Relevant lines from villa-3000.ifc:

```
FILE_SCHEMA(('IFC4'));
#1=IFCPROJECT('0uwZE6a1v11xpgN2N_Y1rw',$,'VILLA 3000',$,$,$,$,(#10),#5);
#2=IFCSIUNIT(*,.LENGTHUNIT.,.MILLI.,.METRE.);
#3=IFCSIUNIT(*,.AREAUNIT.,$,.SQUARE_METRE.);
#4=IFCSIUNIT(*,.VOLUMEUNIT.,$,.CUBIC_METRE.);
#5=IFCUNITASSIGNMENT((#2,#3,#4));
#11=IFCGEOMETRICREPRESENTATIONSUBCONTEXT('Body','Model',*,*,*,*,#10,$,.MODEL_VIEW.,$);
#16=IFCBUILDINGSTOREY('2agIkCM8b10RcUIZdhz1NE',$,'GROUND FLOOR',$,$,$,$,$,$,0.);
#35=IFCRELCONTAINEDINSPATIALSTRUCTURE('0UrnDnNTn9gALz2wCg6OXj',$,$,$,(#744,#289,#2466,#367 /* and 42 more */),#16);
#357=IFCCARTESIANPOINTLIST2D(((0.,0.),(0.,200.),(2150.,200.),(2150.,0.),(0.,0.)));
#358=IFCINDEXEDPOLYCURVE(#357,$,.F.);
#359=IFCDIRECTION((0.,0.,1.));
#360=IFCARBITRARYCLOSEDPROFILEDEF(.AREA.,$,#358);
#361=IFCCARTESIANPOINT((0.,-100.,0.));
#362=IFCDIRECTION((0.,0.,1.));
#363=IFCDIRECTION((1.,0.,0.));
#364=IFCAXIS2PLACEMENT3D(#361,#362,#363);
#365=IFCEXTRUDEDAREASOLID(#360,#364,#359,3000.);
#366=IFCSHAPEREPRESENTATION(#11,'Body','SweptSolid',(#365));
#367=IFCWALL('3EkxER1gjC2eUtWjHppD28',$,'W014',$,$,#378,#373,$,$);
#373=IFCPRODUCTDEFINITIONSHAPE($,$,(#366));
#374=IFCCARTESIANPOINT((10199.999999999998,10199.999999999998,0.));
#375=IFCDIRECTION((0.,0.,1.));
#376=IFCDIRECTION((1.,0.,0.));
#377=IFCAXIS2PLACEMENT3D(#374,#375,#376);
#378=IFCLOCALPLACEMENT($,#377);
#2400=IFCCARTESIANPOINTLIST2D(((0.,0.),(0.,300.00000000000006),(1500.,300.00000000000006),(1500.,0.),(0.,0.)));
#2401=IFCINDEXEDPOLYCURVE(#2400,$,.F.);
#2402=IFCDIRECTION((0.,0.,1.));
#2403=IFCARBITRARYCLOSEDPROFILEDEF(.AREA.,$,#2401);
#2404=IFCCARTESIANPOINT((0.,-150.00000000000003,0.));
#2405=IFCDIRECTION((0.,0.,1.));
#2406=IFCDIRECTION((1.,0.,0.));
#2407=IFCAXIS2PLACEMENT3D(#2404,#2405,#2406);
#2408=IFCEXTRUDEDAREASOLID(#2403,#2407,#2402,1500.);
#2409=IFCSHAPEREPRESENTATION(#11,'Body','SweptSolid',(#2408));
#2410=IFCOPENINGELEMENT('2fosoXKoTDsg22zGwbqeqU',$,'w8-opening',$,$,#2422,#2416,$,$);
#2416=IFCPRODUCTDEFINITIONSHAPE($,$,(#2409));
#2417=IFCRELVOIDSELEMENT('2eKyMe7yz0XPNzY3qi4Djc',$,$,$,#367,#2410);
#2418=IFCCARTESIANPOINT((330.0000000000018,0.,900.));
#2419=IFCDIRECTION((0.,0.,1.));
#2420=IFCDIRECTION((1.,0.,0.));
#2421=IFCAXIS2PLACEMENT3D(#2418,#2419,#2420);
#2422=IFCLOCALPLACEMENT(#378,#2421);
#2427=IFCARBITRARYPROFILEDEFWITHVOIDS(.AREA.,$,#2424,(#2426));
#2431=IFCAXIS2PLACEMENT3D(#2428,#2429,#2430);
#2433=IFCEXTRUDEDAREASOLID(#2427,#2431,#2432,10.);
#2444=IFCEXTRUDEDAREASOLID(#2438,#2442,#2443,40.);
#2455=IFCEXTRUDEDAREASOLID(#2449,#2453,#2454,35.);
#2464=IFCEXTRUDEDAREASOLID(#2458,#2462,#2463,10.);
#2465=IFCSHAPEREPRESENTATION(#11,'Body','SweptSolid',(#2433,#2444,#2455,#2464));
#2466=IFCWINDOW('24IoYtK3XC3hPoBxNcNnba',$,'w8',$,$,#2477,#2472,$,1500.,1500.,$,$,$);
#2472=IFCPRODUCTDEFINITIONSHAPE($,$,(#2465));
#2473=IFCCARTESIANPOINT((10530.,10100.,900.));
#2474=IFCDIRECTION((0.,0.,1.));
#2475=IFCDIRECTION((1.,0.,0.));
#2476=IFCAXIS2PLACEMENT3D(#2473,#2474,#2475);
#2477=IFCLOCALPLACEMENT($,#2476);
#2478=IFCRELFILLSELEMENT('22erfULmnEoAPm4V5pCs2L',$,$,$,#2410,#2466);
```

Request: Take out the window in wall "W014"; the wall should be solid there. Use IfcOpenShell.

```python
import ifcopenshell
import ifcopenshell.api.feature
import ifcopenshell.api.root
import ifcopenshell.geom
import ifcopenshell.util.shape

model = ifcopenshell.open("villa-3000.ifc")
settings = ifcopenshell.geom.settings()


def volume(element):
    """Net volume in cubic metres, openings subtracted."""
    shape = ifcopenshell.geom.create_shape(settings, element)
    return ifcopenshell.util.shape.get_volume(shape.geometry)


window = model.by_guid("24IoYtK3XC3hPoBxNcNnba")
opening = window.FillsVoids[0].RelatingOpeningElement
wall = opening.VoidsElements[0].RelatingBuildingElement
before = volume(wall)

ifcopenshell.api.root.remove_product(model, product=window)
ifcopenshell.api.feature.remove_feature(model, feature=opening)

after = volume(wall)

print(f"wall volume {before:.3f} -> {after:.3f} m3")

model.write("villa-3000_updated.ifc")
```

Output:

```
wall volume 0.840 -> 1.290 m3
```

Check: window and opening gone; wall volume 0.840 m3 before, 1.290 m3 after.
